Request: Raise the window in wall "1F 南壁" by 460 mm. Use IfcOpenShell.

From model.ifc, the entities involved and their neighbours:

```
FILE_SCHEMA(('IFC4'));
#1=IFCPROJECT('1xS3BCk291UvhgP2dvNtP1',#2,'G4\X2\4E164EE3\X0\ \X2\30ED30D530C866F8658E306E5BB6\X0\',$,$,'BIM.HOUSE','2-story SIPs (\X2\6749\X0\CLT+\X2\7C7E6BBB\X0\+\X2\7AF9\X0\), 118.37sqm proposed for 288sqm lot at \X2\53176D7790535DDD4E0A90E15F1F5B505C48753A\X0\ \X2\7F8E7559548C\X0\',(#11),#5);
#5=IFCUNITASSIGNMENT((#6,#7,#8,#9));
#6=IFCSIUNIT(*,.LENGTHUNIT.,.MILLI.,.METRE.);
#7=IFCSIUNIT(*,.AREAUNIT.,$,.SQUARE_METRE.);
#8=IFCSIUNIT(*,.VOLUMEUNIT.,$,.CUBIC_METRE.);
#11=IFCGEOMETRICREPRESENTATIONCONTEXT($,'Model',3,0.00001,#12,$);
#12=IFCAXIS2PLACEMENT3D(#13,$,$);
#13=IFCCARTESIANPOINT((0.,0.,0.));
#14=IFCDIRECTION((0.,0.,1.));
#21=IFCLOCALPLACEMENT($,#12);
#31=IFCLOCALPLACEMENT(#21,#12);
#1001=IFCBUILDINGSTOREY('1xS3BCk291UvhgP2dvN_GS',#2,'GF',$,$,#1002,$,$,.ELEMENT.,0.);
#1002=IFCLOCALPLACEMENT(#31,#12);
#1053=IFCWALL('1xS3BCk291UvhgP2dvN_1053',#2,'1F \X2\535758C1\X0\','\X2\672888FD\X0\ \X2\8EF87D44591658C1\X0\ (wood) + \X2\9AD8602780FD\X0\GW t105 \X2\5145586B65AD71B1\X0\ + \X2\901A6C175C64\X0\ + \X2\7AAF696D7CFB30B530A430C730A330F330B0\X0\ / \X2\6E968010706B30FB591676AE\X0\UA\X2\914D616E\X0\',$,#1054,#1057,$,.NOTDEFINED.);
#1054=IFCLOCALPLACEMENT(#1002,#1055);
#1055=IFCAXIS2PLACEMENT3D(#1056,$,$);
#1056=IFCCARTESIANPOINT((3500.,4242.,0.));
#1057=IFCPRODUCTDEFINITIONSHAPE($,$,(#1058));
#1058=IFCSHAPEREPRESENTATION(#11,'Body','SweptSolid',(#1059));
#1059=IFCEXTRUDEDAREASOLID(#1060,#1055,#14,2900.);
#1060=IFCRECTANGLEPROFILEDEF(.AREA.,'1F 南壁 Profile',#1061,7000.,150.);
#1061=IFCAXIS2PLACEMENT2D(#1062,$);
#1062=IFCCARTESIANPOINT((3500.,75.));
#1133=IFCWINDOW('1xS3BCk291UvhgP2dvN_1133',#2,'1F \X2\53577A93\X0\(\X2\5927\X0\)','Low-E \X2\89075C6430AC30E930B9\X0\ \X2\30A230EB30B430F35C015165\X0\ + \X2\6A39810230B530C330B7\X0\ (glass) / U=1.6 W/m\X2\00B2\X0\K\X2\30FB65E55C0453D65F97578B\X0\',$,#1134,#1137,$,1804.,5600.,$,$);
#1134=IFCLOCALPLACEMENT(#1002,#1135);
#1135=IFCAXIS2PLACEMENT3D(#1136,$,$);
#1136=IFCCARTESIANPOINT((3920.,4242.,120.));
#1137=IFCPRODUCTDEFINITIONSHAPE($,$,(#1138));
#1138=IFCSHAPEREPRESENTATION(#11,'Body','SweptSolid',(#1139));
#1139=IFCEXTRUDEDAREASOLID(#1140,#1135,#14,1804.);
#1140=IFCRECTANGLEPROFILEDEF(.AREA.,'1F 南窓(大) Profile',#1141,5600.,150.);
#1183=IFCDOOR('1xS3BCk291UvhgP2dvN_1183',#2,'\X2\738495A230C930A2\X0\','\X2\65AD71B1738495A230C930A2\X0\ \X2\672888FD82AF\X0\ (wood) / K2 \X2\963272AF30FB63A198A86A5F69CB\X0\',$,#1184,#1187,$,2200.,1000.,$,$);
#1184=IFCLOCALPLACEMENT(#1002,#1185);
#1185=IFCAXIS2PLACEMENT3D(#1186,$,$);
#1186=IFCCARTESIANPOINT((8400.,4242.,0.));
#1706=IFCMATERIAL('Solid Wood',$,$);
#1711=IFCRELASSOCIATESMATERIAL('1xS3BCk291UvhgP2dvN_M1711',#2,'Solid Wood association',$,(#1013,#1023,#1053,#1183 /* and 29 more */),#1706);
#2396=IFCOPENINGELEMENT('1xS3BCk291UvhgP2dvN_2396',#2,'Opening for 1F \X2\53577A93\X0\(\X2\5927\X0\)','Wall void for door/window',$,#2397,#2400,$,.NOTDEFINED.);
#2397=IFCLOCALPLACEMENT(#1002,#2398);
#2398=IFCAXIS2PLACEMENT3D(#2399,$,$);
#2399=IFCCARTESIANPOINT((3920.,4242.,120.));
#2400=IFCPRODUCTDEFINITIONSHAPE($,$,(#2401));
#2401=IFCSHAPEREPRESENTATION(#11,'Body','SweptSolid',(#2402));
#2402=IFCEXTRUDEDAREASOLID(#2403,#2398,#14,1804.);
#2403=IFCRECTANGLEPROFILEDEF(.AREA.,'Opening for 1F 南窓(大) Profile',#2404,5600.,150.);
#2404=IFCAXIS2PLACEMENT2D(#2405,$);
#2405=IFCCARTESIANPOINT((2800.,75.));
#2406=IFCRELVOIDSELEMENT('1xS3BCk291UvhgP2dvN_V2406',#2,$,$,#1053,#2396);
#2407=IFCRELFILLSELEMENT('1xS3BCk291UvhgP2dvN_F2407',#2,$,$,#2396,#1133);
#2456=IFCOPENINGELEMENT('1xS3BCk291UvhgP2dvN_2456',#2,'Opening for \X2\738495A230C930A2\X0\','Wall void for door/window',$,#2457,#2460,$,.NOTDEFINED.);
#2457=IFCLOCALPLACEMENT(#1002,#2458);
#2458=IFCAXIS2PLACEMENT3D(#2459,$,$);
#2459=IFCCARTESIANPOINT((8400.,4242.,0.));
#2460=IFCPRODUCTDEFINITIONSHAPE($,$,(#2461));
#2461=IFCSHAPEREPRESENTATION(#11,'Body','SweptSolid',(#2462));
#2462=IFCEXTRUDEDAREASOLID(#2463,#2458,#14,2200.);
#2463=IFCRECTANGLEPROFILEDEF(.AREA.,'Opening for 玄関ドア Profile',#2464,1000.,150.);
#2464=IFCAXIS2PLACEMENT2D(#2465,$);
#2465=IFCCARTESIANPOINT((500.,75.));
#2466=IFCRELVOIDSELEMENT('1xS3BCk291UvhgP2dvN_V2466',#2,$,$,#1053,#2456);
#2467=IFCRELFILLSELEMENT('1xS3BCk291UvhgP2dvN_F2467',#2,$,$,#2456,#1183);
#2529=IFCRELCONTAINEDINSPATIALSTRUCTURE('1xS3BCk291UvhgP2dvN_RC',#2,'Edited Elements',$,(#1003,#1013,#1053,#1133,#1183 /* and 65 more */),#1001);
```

```python
import numpy as np
import ifcopenshell
import ifcopenshell.api.geometry
import ifcopenshell.util.placement
import ifcopenshell.util.unit

model = ifcopenshell.open("model.ifc")
unit_scale = ifcopenshell.util.unit.calculate_unit_scale(model)

window = model.by_guid("1xS3BCk291UvhgP2dvN_1133")
opening = window.FillsVoids[0].RelatingOpeningElement
dz = 0.46 / unit_scale

shift = np.array([0.0, 0.0, dz])
# The window is not placed relative to its opening, so move both.
for product in (opening, window):
    matrix = ifcopenshell.util.placement.get_local_placement(product.ObjectPlacement)
    matrix[:3, 3] += shift
    ifcopenshell.api.geometry.edit_object_placement(model, product=product, matrix=matrix, is_si=False)

print(f"moved by {dz * unit_scale:+.3f} m")

model.write("model-out.ifc")
```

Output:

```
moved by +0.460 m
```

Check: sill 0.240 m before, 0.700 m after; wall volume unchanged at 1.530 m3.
